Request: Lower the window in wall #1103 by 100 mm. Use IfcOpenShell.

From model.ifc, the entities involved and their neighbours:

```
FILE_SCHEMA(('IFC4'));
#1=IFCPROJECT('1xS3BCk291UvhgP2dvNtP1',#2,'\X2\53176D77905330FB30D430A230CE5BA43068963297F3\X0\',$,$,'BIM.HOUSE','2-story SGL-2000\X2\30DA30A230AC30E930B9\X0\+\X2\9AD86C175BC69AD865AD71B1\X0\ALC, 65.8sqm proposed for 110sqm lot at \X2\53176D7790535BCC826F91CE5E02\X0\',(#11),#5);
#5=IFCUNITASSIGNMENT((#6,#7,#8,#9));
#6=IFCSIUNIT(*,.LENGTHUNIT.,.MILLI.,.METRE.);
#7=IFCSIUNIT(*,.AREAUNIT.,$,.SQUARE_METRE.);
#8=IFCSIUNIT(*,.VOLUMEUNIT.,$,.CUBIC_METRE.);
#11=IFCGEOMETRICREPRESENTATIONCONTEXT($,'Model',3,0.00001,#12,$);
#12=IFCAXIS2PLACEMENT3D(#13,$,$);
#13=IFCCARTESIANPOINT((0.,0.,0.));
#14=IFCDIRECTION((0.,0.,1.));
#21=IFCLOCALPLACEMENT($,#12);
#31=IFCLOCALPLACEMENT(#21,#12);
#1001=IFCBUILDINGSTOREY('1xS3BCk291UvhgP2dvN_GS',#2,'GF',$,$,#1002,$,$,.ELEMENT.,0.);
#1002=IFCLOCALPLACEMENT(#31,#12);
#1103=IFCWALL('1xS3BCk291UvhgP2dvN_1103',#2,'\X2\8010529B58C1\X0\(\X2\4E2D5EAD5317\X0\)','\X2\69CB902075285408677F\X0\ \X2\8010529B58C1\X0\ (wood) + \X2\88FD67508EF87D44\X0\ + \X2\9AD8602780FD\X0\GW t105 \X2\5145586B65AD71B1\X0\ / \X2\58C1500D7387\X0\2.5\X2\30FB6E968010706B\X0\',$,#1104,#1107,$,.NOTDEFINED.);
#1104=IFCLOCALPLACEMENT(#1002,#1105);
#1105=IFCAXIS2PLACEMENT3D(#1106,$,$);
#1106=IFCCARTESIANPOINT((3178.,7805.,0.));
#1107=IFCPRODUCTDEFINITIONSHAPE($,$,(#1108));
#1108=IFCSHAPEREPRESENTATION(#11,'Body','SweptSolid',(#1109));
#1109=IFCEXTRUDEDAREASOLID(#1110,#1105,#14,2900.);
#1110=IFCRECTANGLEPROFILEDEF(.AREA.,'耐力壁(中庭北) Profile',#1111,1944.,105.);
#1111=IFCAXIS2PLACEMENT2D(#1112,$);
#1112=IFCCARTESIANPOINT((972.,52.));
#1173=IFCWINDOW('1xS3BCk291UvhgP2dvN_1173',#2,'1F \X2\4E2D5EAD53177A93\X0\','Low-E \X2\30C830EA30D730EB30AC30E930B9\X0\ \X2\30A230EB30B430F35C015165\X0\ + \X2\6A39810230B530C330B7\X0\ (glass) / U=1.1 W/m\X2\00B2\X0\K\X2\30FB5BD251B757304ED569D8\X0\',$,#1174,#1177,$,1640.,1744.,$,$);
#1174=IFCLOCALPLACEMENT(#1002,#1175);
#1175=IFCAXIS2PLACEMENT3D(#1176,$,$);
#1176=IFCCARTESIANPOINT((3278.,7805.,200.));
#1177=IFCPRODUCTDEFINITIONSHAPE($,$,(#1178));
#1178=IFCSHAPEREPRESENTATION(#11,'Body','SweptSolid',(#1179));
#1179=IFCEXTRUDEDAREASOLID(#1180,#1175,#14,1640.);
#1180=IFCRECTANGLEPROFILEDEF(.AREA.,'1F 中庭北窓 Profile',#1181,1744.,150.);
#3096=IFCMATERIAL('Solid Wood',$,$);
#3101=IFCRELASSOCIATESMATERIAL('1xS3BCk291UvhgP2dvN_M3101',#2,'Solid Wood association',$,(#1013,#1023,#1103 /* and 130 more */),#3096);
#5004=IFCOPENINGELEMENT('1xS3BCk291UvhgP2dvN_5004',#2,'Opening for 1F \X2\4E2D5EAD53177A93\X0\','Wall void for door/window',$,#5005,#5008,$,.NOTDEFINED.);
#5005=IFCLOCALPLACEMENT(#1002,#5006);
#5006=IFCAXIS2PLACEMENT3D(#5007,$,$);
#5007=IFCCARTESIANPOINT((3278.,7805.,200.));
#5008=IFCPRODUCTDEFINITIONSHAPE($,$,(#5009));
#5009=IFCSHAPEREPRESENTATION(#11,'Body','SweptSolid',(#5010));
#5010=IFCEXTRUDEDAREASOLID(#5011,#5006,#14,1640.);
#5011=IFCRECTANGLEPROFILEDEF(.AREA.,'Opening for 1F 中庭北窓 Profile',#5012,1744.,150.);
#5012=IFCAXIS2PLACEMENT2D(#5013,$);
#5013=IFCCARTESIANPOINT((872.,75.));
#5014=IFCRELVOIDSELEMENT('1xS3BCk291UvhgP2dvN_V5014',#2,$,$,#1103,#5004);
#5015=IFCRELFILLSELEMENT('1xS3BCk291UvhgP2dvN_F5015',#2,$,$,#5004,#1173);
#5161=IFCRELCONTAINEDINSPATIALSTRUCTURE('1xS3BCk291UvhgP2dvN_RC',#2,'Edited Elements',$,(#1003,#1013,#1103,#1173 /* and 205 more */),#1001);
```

```python
import numpy as np
import ifcopenshell
import ifcopenshell.api.geometry
import ifcopenshell.util.placement
import ifcopenshell.util.unit

model = ifcopenshell.open("model.ifc")
unit_scale = ifcopenshell.util.unit.calculate_unit_scale(model)

window = model.by_id(1173)
opening = window.FillsVoids[0].RelatingOpeningElement
dz = -0.1 / unit_scale

shift = np.array([0.0, 0.0, dz])
# The window is not placed relative to its opening, so move both.
for product in (opening, window):
    matrix = ifcopenshell.util.placement.get_local_placement(product.ObjectPlacement)
    matrix[:3, 3] += shift
    ifcopenshell.api.geometry.edit_object_placement(model, product=product, matrix=matrix, is_si=False)

print(f"moved by {dz * unit_scale:+.3f} m")

model.write("model_v2.ifc")
```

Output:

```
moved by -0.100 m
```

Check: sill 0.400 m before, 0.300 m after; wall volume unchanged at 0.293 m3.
